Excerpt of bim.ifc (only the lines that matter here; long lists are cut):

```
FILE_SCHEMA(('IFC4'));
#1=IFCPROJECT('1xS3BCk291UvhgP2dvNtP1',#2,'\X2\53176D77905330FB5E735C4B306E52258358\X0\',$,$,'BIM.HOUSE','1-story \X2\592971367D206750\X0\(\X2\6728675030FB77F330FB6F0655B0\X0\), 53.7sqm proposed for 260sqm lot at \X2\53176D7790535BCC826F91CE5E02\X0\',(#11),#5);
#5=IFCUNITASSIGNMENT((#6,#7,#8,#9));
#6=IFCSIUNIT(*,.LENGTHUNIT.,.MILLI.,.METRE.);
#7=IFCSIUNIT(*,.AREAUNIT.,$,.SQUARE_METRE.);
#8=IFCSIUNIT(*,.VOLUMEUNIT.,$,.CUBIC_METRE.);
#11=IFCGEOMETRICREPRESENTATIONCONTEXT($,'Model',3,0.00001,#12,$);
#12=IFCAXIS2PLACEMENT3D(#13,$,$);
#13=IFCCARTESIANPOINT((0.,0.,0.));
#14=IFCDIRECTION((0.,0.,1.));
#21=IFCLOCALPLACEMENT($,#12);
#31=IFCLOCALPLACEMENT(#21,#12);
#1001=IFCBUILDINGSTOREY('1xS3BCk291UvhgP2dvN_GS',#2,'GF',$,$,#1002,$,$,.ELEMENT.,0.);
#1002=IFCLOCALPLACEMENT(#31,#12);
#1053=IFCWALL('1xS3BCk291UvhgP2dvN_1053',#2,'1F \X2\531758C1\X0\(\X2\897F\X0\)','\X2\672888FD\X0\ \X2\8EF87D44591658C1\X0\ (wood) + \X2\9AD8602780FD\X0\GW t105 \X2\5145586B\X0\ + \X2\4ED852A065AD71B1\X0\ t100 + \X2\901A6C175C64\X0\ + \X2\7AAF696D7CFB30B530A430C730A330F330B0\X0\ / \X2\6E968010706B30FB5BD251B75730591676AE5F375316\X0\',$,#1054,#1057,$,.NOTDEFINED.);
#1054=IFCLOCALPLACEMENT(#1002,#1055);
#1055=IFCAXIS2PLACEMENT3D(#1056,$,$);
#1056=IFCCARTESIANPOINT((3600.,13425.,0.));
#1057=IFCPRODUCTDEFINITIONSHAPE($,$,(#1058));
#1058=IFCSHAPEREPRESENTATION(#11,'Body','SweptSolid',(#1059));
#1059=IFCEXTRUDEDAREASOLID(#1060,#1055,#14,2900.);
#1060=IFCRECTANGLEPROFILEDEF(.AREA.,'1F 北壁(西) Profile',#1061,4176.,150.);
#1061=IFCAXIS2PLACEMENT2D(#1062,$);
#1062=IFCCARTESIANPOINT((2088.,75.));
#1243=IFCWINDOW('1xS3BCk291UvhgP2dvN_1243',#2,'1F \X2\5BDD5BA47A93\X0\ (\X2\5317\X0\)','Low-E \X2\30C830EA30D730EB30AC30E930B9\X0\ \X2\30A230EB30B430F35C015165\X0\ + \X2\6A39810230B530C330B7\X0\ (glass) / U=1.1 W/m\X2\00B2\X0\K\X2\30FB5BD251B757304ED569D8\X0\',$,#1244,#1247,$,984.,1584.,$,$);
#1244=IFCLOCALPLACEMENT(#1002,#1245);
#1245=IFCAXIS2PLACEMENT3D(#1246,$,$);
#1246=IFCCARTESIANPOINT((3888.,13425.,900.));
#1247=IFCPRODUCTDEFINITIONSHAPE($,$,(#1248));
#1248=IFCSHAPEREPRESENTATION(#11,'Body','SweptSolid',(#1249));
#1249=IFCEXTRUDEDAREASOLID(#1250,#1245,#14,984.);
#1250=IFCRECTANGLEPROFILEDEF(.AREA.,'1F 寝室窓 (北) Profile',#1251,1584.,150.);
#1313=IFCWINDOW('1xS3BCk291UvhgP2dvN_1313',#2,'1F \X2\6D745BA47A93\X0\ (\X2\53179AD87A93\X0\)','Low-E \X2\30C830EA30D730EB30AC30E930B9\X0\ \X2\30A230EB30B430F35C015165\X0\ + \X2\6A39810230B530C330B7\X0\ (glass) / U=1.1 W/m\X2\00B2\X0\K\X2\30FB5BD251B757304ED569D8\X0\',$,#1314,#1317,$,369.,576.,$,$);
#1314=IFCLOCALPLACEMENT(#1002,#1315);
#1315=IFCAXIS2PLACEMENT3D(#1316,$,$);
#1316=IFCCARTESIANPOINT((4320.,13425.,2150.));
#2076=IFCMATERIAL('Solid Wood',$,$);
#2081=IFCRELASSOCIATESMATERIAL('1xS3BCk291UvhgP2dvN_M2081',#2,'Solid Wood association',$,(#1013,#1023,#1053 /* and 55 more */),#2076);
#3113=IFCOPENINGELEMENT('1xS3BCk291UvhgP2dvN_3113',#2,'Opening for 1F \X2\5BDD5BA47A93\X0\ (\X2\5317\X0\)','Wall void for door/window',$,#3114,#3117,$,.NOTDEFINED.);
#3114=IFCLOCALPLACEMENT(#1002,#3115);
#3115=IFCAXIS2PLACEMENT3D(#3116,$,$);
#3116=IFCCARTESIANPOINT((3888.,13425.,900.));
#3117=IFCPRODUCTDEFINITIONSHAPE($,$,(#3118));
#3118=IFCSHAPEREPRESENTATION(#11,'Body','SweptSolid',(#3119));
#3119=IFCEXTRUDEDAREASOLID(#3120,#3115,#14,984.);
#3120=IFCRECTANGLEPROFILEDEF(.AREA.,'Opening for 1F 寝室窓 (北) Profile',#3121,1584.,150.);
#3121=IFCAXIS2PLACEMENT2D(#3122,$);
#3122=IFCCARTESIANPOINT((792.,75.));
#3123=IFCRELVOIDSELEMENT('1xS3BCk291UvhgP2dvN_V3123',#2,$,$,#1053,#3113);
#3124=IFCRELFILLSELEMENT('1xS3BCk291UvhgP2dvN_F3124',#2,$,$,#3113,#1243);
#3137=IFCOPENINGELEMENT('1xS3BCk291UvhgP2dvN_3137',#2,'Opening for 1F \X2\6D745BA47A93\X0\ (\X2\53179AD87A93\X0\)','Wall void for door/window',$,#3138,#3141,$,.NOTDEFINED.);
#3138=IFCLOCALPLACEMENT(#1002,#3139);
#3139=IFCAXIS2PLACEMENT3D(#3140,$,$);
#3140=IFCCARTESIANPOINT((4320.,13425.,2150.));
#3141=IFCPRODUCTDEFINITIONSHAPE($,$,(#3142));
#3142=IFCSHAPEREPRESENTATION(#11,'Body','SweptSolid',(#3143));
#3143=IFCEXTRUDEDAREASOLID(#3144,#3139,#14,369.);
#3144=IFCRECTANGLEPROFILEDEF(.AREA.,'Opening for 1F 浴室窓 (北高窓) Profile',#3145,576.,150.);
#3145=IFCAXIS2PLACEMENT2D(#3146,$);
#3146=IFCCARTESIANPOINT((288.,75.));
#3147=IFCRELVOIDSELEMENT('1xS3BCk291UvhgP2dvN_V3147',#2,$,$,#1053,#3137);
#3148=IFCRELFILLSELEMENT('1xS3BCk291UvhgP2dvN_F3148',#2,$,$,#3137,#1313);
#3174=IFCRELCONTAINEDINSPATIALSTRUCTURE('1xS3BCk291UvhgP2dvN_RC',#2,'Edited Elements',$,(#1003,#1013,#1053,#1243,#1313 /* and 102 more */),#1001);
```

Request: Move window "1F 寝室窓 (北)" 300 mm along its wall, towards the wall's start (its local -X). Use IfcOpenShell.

```python
import ifcopenshell
import ifcopenshell.api.geometry
import ifcopenshell.util.placement
import ifcopenshell.util.unit

model = ifcopenshell.open("bim.ifc")
unit_scale = ifcopenshell.util.unit.calculate_unit_scale(model)

window = model.by_guid("1xS3BCk291UvhgP2dvN_1243")
opening = window.FillsVoids[0].RelatingOpeningElement
wall = opening.VoidsElements[0].RelatingBuildingElement

wall_matrix = ifcopenshell.util.placement.get_local_placement(wall.ObjectPlacement)
shift = wall_matrix[:3, 0] * -0.3 / unit_scale
before = ifcopenshell.util.placement.get_local_placement(window.ObjectPlacement)[:3, 3].copy()

# The window is not placed relative to its opening, so move both.
for product in (opening, window):
    matrix = ifcopenshell.util.placement.get_local_placement(product.ObjectPlacement)
    matrix[:3, 3] += shift
    ifcopenshell.api.geometry.edit_object_placement(model, product=product, matrix=matrix, is_si=False)

after = ifcopenshell.util.placement.get_local_placement(window.ObjectPlacement)[:3, 3]
print("window moved by", (after - before).round(3) + 0.0)

model.write("bim_rev.ifc")
```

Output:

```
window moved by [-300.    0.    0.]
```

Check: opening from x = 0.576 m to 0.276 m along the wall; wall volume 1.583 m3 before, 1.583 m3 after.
